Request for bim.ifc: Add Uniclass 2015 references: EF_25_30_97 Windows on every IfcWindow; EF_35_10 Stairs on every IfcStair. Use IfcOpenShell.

First a look at what the model holds.

```python
import ifcopenshell

model = ifcopenshell.open("bim.ifc")
print(model.schema)
print("classifications:", [c.Name for c in model.by_type("IfcClassification")])
for ifc_class in ("IfcDoor", "IfcRoof", "IfcStair", "IfcWall", "IfcWindow"):
    print(ifc_class, len(model.by_type(ifc_class)))
```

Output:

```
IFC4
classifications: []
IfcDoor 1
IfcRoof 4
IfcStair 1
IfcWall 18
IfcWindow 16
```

```python
import ifcopenshell
import ifcopenshell.api.classification

model = ifcopenshell.open("bim.ifc")

system = ifcopenshell.api.classification.add_classification(model, classification="Uniclass 2015")

codes = {
    "IfcWindow": ("EF_25_30_97", "Windows"),
    "IfcStair": ("EF_35_10", "Stairs"),
}
for ifc_class, (code, name) in codes.items():
    products = model.by_type(ifc_class)
    ifcopenshell.api.classification.add_reference(
        model, products=products, classification=system, identification=code, name=name
    )
    print(code, len(products))

model.write("bim_v2.ifc")
```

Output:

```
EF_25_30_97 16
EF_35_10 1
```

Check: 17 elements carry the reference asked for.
